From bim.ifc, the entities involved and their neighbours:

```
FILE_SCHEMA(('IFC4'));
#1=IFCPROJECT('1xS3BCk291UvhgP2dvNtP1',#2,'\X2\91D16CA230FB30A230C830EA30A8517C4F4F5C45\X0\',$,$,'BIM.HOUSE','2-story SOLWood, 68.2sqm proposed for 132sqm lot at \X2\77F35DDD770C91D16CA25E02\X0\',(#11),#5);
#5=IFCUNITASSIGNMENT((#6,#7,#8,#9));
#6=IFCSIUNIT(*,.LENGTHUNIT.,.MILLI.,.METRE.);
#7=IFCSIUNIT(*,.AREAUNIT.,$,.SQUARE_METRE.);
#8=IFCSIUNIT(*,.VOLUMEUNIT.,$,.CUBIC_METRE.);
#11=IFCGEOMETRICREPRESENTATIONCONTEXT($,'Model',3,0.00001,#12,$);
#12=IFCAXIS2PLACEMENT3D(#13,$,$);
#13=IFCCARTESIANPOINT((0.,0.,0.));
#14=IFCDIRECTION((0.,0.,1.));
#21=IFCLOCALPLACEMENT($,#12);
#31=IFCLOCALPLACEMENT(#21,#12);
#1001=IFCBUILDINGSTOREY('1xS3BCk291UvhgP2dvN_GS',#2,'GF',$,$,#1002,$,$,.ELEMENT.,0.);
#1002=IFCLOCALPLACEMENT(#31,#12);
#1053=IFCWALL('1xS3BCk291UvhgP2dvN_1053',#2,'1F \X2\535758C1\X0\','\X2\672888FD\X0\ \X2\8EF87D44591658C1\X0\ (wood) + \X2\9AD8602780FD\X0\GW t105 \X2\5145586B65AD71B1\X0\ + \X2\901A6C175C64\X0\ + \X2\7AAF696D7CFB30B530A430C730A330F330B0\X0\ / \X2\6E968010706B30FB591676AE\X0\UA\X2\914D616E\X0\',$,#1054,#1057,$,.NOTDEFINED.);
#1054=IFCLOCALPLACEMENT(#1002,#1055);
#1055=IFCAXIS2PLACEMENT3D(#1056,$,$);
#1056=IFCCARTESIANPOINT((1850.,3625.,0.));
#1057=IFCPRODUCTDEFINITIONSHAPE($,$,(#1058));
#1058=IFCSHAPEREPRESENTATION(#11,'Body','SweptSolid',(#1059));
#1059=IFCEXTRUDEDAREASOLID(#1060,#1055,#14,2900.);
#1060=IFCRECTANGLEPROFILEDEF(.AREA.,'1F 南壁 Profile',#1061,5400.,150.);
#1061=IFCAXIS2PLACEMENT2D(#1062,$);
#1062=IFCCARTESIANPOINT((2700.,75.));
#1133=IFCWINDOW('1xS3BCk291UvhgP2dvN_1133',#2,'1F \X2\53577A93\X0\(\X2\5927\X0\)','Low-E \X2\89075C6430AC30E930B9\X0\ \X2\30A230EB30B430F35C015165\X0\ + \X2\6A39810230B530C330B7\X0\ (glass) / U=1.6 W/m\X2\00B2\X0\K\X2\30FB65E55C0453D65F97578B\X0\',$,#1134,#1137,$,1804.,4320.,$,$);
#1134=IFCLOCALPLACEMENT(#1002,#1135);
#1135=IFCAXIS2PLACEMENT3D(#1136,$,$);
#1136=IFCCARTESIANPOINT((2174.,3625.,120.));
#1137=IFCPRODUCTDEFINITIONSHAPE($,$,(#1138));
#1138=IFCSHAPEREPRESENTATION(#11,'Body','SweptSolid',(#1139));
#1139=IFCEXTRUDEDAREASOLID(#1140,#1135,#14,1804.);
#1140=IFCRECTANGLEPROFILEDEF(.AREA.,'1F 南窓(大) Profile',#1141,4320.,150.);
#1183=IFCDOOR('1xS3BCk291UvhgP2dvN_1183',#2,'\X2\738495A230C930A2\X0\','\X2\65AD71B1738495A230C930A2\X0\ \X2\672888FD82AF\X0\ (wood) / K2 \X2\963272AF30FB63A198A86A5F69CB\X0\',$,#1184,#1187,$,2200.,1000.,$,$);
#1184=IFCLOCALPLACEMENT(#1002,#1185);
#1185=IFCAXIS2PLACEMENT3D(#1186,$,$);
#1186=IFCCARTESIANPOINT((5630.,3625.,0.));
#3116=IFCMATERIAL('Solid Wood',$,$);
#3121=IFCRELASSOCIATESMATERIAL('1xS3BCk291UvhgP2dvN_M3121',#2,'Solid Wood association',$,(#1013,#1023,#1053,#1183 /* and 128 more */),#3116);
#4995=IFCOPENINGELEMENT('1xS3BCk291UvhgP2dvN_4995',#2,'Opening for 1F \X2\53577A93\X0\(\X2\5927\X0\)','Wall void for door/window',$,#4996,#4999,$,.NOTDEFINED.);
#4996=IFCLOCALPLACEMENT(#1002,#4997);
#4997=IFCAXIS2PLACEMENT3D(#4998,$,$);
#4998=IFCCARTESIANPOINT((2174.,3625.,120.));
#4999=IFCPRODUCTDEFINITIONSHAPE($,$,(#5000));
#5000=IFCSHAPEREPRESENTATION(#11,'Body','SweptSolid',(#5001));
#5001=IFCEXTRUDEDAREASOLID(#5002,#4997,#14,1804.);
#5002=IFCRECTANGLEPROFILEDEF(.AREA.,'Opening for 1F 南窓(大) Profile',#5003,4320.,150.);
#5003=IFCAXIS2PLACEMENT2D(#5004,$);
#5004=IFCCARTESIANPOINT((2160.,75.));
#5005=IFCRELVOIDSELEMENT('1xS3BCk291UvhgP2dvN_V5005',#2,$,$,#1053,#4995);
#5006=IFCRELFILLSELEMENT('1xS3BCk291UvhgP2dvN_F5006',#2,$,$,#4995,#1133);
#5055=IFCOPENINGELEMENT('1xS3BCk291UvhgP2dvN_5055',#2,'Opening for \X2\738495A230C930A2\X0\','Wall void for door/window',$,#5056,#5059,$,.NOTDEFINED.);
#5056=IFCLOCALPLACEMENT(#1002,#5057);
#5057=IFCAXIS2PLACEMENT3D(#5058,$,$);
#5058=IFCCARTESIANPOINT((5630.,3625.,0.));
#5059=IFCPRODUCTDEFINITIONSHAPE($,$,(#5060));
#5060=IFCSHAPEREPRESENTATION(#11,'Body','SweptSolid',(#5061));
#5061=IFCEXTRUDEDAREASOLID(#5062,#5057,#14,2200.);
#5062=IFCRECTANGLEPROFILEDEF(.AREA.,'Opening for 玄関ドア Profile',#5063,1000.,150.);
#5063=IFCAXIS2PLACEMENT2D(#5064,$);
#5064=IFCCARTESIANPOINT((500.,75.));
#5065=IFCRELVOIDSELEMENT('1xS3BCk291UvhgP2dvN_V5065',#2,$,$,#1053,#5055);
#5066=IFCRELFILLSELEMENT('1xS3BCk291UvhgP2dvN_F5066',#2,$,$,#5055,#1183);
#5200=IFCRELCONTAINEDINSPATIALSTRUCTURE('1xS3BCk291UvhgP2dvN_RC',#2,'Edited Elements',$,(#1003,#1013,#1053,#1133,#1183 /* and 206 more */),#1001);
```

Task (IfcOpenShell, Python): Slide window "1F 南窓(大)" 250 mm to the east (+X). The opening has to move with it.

```python
import ifcopenshell
import ifcopenshell.api.geometry
import ifcopenshell.util.placement
import ifcopenshell.util.unit

model = ifcopenshell.open("bim.ifc")
unit_scale = ifcopenshell.util.unit.calculate_unit_scale(model)

window = model.by_guid("1xS3BCk291UvhgP2dvN_1133")
opening = window.FillsVoids[0].RelatingOpeningElement
wall = opening.VoidsElements[0].RelatingBuildingElement

wall_matrix = ifcopenshell.util.placement.get_local_placement(wall.ObjectPlacement)
shift = wall_matrix[:3, 0] * 0.25 / unit_scale
before = ifcopenshell.util.placement.get_local_placement(window.ObjectPlacement)[:3, 3].copy()

# The window is not placed relative to its opening, so move both.
for product in (opening, window):
    matrix = ifcopenshell.util.placement.get_local_placement(product.ObjectPlacement)
    matrix[:3, 3] += shift
    ifcopenshell.api.geometry.edit_object_placement(model, product=product, matrix=matrix, is_si=False)

after = ifcopenshell.util.placement.get_local_placement(window.ObjectPlacement)[:3, 3]
print("window moved by", (after - before).round(3) + 0.0)

model.write("bim-out.ifc")
```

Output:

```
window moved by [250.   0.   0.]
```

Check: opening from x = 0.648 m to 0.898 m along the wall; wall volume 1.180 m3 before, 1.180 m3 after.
